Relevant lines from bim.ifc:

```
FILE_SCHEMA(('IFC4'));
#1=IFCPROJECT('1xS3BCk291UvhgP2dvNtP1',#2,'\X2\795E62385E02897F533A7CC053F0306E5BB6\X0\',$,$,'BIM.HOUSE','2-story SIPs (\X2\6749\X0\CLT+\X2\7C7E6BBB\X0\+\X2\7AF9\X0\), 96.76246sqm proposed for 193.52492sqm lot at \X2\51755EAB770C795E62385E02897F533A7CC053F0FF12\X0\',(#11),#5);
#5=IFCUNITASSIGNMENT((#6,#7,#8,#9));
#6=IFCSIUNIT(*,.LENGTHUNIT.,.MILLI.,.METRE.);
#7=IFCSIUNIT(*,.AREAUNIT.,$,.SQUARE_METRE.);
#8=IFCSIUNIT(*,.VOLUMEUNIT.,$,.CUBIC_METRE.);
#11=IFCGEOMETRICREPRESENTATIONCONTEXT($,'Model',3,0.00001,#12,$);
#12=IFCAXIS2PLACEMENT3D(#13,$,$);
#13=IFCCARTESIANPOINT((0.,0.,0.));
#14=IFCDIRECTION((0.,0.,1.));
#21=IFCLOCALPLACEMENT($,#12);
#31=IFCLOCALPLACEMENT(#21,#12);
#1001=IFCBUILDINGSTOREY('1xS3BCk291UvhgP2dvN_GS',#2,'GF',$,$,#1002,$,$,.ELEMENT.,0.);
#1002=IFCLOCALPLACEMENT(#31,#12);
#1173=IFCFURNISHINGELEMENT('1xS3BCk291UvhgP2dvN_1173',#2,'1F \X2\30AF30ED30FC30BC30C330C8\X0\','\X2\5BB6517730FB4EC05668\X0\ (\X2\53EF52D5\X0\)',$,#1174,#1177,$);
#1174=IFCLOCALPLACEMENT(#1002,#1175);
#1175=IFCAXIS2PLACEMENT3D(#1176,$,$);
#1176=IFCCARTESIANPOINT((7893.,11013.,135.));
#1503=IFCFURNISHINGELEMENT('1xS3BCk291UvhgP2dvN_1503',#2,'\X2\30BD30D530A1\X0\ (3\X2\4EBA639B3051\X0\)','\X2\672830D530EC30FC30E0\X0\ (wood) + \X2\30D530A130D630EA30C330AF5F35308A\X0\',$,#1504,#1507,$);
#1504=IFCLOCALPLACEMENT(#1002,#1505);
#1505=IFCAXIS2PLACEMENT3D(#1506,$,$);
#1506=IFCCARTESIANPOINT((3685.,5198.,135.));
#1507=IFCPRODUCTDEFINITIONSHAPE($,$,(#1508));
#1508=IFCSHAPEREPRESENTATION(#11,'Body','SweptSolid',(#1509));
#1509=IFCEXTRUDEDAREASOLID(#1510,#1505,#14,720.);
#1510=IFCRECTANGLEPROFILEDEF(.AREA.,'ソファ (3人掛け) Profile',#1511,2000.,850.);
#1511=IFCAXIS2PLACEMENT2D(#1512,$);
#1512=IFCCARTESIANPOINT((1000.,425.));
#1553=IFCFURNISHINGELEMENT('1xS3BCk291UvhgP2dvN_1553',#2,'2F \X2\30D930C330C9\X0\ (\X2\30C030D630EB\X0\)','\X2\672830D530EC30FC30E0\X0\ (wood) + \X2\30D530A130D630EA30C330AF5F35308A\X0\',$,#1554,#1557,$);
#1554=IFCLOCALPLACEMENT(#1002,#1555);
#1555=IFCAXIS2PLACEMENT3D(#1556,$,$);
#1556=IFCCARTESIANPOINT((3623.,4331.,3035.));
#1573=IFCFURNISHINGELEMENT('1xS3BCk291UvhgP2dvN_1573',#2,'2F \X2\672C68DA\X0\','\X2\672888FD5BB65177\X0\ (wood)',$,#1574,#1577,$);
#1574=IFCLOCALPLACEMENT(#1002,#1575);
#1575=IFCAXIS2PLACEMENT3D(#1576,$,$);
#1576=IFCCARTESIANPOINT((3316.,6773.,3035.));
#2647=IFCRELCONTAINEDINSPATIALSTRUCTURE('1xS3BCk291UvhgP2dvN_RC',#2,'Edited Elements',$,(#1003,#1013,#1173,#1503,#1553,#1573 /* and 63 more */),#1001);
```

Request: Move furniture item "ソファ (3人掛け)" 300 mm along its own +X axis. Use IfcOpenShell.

```python
import ifcopenshell
import ifcopenshell.api.geometry
import ifcopenshell.util.placement

model = ifcopenshell.open("bim.ifc")

item = model.by_guid("1xS3BCk291UvhgP2dvN_1503")
matrix = ifcopenshell.util.placement.get_local_placement(item.ObjectPlacement)
matrix[:3, 3] += matrix[:3, 0] * 300.0
ifcopenshell.api.geometry.edit_object_placement(model, product=item, matrix=matrix, is_si=False)

print(ifcopenshell.util.placement.get_local_placement(item.ObjectPlacement).round(3) + 0.0)

model.write("bim_rev.ifc")
```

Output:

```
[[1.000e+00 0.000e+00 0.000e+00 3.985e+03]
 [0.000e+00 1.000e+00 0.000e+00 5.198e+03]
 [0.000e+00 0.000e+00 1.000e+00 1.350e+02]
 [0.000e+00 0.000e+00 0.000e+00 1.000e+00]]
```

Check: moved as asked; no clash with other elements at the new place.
